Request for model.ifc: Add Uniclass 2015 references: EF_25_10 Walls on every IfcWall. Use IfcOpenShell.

First a look at what the model holds.

```python
import ifcopenshell

model = ifcopenshell.open("model.ifc")
print(model.schema)
print("classifications:", [c.Name for c in model.by_type("IfcClassification")])
for ifc_class in ("IfcDoor", "IfcRoof", "IfcStair", "IfcWall", "IfcWindow"):
    print(ifc_class, len(model.by_type(ifc_class)))
```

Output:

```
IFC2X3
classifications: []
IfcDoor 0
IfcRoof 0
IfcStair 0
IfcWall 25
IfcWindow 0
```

```python
import ifcopenshell
import ifcopenshell.api.classification

model = ifcopenshell.open("model.ifc")

# IFC2X3 requires Source and Edition and has no link from the project to the system.
system = model.create_entity("IfcClassification", Source="NBS", Edition="2015", Name="Uniclass 2015")

codes = {
    "IfcWall": ("EF_25_10", "Walls"),
}
for ifc_class, (code, name) in codes.items():
    products = model.by_type(ifc_class)
    ifcopenshell.api.classification.add_reference(
        model, products=products, classification=system, identification=code, name=name
    )
    print(code, len(products))

model.write("model_rev.ifc")
```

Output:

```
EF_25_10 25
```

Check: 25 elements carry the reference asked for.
